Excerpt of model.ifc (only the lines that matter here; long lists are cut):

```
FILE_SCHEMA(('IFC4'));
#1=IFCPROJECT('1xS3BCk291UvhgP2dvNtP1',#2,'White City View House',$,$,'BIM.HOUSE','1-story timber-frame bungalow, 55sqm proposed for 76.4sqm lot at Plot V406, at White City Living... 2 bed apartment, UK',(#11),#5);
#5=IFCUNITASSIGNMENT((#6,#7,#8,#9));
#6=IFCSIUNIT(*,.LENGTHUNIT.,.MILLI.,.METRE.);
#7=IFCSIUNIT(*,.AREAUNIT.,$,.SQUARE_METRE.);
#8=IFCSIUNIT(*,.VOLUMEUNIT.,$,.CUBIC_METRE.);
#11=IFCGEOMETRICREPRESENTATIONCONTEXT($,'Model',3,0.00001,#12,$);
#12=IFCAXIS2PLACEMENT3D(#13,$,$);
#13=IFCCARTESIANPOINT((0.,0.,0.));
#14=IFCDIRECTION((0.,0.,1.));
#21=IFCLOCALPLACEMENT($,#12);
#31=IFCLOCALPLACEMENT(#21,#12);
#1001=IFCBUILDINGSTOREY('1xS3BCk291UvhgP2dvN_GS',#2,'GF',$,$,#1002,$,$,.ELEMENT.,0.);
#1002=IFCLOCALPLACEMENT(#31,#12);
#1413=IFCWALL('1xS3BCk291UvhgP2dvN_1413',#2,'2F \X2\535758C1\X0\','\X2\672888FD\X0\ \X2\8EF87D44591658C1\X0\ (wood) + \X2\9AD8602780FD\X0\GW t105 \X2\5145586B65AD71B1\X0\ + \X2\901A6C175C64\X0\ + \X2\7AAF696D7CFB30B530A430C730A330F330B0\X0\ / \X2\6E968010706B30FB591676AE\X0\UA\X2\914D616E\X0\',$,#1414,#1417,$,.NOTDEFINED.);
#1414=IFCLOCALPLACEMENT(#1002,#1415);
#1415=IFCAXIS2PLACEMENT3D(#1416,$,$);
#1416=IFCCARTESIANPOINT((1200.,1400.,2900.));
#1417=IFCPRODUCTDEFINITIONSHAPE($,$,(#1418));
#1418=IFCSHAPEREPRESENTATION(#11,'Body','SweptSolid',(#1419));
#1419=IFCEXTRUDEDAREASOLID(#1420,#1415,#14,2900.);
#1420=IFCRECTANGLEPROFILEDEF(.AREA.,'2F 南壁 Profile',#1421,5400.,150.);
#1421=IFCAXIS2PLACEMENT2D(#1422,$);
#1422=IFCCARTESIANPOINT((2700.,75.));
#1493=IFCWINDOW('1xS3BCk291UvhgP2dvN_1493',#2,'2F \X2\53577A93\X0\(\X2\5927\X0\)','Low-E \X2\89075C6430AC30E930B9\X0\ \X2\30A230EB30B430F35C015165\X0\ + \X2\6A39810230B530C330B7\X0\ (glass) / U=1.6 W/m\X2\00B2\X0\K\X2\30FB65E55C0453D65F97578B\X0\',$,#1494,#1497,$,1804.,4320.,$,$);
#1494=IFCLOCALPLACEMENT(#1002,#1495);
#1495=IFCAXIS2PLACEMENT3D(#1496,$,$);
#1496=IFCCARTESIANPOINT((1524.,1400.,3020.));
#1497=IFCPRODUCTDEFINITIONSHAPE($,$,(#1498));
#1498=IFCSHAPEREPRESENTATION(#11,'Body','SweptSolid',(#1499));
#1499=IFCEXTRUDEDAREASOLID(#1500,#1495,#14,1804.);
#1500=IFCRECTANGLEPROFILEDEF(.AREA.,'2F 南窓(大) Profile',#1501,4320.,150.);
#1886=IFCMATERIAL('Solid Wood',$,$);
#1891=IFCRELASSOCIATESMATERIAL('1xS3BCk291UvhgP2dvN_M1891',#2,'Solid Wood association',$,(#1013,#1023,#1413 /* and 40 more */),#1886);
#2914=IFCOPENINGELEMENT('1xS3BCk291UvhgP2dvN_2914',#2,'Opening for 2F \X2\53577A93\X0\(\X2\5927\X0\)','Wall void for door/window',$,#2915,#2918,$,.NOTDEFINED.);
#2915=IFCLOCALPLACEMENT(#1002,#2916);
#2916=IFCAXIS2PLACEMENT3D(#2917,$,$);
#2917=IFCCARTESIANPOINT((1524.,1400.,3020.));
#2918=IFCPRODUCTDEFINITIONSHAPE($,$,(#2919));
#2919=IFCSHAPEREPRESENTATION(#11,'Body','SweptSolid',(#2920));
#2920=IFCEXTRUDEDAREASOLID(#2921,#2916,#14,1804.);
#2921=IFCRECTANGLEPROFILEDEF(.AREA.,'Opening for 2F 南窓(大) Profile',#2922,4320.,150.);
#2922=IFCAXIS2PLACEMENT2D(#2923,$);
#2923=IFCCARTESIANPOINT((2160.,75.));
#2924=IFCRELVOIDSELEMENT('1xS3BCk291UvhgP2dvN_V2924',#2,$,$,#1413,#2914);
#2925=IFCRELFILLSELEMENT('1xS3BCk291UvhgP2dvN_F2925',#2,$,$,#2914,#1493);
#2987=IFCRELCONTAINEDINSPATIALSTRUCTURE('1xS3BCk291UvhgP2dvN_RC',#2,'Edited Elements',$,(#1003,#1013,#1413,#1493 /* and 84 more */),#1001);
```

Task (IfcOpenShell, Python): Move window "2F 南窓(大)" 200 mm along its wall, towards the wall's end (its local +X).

```python
import ifcopenshell
import ifcopenshell.api.geometry
import ifcopenshell.util.placement
import ifcopenshell.util.unit

model = ifcopenshell.open("model.ifc")
unit_scale = ifcopenshell.util.unit.calculate_unit_scale(model)

window = model.by_guid("1xS3BCk291UvhgP2dvN_1493")
opening = window.FillsVoids[0].RelatingOpeningElement
wall = opening.VoidsElements[0].RelatingBuildingElement

wall_matrix = ifcopenshell.util.placement.get_local_placement(wall.ObjectPlacement)
shift = wall_matrix[:3, 0] * 0.2 / unit_scale
before = ifcopenshell.util.placement.get_local_placement(window.ObjectPlacement)[:3, 3].copy()

# The window is not placed relative to its opening, so move both.
for product in (opening, window):
    matrix = ifcopenshell.util.placement.get_local_placement(product.ObjectPlacement)
    matrix[:3, 3] += shift
    ifcopenshell.api.geometry.edit_object_placement(model, product=product, matrix=matrix, is_si=False)

after = ifcopenshell.util.placement.get_local_placement(window.ObjectPlacement)[:3, 3]
print("window moved by", (after - before).round(3) + 0.0)

model.write("model_updated.ifc")
```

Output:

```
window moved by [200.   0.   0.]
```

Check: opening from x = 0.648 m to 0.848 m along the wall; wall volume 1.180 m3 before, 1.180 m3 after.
